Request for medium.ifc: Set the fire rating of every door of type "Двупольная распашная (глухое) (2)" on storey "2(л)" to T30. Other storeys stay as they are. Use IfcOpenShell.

First a look at what the model holds.

```python
import ifcopenshell
import ifcopenshell.util.element

model = ifcopenshell.open("medium.ifc")
print(model.schema)
storey = next(s for s in model.by_type("IfcBuildingStorey") if s.Name == "2(л)")
doors = [e for e in ifcopenshell.util.element.get_decomposition(storey) if e.is_a("IfcDoor")]
seen = {}
for e in doors:
    element_type = ifcopenshell.util.element.get_type(e)
    key = (element_type.Name if element_type != e and element_type else None, ifcopenshell.util.element.get_pset(e, "Pset_DoorCommon", "FireRating"))
    seen[key] = seen.get(key, 0) + 1
for (name, value), count in sorted(seen.items(), key=str):
    print(count, "x", name, "|", value)
```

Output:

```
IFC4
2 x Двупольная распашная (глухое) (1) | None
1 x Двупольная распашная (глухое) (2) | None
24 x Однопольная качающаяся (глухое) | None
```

```python
import ifcopenshell
import ifcopenshell.api.pset
import ifcopenshell.util.element

model = ifcopenshell.open("medium.ifc")

storey = next(s for s in model.by_type("IfcBuildingStorey") if s.Name == "2(л)")
doors = [e for e in ifcopenshell.util.element.get_decomposition(storey) if e.is_a("IfcDoor")]

count = 0
for e in doors:
    element_type = ifcopenshell.util.element.get_type(e)
    if element_type in (None, e) or element_type.Name != "Двупольная распашная (глухое) (2)":
        continue
    # add_pset returns the element's existing set when there is one.
    pset = ifcopenshell.api.pset.add_pset(model, product=e, name="Pset_DoorCommon")
    ifcopenshell.api.pset.edit_pset(model, pset=pset, properties={"FireRating": "T30"})
    count += 1

print(count, "doors updated")

model.write("medium_edited.ifc")
```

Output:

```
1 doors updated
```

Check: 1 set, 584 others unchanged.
